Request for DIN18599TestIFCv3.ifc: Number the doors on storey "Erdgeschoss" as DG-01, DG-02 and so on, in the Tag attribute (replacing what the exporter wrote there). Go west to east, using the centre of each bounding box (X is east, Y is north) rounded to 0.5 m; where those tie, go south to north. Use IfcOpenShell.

First a look at what the model holds.

```python
import ifcopenshell
import ifcopenshell.util.element
import ifcopenshell.util.placement

model = ifcopenshell.open("DIN18599TestIFCv3.ifc")
print(model.schema)
storey = next(s for s in model.by_type("IfcBuildingStorey") if s.Name == "Erdgeschoss")
doors = [e for e in ifcopenshell.util.element.get_decomposition(storey) if e.is_a("IfcDoor")]
for e in sorted(doors, key=lambda e: e.id()):
    origin = ifcopenshell.util.placement.get_local_placement(e.ObjectPlacement)[:3, 3]
    print(e.id(), e.Tag, e.Name, origin.round(2) + 0.0, sep=" | ")
```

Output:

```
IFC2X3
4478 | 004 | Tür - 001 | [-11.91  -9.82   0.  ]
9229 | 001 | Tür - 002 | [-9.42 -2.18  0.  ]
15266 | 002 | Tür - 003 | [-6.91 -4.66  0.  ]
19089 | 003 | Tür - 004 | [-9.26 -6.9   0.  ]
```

```python
import ifcopenshell
import ifcopenshell.geom
import ifcopenshell.util.element
import ifcopenshell.util.shape

model = ifcopenshell.open("DIN18599TestIFCv3.ifc")
settings = ifcopenshell.geom.settings()
settings.set("use-world-coords", True)


def centre(element):
    shape = ifcopenshell.geom.create_shape(settings, element)
    return ifcopenshell.util.shape.get_bbox_centroid(shape.geometry)


storey = next(s for s in model.by_type("IfcBuildingStorey") if s.Name == "Erdgeschoss")
doors = [e for e in ifcopenshell.util.element.get_decomposition(storey) if e.is_a("IfcDoor")]

# Insertion points can sit at a corner or the storey origin, so sort by the geometry (in metres).
centres = {e: centre(e) for e in doors}
doors.sort(key=lambda e: (round(centres[e][0] / 0.5), centres[e][1]))

for i, e in enumerate(doors, start=1):
    number = f"DG-{i:02d}"
    e.Tag = number
    print(e.id(), number)

model.write("DIN18599TestIFCv3_rev.ifc")
```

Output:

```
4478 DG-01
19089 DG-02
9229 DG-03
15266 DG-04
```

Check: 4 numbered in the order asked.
